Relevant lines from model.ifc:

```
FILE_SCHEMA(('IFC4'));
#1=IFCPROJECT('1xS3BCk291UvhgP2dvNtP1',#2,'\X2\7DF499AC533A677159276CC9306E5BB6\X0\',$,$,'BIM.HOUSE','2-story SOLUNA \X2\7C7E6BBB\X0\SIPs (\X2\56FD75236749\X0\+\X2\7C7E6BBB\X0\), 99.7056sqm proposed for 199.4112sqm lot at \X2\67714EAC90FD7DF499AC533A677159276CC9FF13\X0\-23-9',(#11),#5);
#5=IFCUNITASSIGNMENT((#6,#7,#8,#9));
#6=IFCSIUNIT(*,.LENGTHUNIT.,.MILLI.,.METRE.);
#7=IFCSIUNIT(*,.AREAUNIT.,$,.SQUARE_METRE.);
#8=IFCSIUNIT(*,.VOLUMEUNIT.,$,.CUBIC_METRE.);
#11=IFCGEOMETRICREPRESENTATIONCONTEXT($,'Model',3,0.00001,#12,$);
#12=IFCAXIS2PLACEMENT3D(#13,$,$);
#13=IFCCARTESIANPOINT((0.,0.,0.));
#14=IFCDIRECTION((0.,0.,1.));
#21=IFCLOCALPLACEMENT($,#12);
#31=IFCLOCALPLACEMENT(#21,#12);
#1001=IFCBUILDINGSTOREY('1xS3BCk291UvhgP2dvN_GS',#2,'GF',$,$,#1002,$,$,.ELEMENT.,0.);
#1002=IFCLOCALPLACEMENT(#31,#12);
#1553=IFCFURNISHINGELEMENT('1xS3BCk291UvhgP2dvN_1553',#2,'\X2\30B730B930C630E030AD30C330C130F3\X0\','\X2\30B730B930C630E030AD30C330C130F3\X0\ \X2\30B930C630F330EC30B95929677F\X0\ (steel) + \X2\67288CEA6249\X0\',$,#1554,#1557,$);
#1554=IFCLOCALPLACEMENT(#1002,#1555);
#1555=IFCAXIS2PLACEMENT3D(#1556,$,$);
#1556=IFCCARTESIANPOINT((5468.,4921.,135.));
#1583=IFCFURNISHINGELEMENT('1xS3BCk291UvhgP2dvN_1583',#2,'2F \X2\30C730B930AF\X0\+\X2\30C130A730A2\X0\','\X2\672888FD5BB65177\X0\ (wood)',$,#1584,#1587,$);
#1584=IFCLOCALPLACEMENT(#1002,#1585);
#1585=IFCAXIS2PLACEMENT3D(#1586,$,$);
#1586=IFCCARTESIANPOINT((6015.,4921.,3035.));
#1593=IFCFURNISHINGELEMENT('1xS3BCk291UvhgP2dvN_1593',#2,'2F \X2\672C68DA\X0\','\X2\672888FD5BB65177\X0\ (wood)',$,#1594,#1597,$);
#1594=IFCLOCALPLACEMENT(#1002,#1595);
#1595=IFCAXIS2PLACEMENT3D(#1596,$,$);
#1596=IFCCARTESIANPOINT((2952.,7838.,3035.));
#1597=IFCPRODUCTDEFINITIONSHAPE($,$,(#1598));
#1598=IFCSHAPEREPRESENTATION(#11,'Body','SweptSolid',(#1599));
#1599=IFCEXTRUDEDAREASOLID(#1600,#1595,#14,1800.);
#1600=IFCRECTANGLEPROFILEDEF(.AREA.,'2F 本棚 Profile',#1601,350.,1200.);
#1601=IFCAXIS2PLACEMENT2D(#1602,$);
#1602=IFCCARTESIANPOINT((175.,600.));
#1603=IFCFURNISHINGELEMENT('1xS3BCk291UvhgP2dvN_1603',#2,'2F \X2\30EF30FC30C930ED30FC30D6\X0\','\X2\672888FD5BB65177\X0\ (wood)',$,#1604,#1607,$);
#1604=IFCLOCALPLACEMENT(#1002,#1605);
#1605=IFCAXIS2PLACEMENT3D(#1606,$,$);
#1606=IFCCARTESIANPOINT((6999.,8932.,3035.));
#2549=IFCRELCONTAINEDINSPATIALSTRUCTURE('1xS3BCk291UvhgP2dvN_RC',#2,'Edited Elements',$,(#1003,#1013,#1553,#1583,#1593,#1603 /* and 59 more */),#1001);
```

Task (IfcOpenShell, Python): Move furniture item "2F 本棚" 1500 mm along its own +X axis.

```python
import ifcopenshell
import ifcopenshell.api.geometry
import ifcopenshell.util.placement

model = ifcopenshell.open("model.ifc")

item = model.by_guid("1xS3BCk291UvhgP2dvN_1593")
matrix = ifcopenshell.util.placement.get_local_placement(item.ObjectPlacement)
matrix[:3, 3] += matrix[:3, 0] * 1500.0
ifcopenshell.api.geometry.edit_object_placement(model, product=item, matrix=matrix, is_si=False)

print(ifcopenshell.util.placement.get_local_placement(item.ObjectPlacement).round(3) + 0.0)

model.write("model_rev.ifc")
```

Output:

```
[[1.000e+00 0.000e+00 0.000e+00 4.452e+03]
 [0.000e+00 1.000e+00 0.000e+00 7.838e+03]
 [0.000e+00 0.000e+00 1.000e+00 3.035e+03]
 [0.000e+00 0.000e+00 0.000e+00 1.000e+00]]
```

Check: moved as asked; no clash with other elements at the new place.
